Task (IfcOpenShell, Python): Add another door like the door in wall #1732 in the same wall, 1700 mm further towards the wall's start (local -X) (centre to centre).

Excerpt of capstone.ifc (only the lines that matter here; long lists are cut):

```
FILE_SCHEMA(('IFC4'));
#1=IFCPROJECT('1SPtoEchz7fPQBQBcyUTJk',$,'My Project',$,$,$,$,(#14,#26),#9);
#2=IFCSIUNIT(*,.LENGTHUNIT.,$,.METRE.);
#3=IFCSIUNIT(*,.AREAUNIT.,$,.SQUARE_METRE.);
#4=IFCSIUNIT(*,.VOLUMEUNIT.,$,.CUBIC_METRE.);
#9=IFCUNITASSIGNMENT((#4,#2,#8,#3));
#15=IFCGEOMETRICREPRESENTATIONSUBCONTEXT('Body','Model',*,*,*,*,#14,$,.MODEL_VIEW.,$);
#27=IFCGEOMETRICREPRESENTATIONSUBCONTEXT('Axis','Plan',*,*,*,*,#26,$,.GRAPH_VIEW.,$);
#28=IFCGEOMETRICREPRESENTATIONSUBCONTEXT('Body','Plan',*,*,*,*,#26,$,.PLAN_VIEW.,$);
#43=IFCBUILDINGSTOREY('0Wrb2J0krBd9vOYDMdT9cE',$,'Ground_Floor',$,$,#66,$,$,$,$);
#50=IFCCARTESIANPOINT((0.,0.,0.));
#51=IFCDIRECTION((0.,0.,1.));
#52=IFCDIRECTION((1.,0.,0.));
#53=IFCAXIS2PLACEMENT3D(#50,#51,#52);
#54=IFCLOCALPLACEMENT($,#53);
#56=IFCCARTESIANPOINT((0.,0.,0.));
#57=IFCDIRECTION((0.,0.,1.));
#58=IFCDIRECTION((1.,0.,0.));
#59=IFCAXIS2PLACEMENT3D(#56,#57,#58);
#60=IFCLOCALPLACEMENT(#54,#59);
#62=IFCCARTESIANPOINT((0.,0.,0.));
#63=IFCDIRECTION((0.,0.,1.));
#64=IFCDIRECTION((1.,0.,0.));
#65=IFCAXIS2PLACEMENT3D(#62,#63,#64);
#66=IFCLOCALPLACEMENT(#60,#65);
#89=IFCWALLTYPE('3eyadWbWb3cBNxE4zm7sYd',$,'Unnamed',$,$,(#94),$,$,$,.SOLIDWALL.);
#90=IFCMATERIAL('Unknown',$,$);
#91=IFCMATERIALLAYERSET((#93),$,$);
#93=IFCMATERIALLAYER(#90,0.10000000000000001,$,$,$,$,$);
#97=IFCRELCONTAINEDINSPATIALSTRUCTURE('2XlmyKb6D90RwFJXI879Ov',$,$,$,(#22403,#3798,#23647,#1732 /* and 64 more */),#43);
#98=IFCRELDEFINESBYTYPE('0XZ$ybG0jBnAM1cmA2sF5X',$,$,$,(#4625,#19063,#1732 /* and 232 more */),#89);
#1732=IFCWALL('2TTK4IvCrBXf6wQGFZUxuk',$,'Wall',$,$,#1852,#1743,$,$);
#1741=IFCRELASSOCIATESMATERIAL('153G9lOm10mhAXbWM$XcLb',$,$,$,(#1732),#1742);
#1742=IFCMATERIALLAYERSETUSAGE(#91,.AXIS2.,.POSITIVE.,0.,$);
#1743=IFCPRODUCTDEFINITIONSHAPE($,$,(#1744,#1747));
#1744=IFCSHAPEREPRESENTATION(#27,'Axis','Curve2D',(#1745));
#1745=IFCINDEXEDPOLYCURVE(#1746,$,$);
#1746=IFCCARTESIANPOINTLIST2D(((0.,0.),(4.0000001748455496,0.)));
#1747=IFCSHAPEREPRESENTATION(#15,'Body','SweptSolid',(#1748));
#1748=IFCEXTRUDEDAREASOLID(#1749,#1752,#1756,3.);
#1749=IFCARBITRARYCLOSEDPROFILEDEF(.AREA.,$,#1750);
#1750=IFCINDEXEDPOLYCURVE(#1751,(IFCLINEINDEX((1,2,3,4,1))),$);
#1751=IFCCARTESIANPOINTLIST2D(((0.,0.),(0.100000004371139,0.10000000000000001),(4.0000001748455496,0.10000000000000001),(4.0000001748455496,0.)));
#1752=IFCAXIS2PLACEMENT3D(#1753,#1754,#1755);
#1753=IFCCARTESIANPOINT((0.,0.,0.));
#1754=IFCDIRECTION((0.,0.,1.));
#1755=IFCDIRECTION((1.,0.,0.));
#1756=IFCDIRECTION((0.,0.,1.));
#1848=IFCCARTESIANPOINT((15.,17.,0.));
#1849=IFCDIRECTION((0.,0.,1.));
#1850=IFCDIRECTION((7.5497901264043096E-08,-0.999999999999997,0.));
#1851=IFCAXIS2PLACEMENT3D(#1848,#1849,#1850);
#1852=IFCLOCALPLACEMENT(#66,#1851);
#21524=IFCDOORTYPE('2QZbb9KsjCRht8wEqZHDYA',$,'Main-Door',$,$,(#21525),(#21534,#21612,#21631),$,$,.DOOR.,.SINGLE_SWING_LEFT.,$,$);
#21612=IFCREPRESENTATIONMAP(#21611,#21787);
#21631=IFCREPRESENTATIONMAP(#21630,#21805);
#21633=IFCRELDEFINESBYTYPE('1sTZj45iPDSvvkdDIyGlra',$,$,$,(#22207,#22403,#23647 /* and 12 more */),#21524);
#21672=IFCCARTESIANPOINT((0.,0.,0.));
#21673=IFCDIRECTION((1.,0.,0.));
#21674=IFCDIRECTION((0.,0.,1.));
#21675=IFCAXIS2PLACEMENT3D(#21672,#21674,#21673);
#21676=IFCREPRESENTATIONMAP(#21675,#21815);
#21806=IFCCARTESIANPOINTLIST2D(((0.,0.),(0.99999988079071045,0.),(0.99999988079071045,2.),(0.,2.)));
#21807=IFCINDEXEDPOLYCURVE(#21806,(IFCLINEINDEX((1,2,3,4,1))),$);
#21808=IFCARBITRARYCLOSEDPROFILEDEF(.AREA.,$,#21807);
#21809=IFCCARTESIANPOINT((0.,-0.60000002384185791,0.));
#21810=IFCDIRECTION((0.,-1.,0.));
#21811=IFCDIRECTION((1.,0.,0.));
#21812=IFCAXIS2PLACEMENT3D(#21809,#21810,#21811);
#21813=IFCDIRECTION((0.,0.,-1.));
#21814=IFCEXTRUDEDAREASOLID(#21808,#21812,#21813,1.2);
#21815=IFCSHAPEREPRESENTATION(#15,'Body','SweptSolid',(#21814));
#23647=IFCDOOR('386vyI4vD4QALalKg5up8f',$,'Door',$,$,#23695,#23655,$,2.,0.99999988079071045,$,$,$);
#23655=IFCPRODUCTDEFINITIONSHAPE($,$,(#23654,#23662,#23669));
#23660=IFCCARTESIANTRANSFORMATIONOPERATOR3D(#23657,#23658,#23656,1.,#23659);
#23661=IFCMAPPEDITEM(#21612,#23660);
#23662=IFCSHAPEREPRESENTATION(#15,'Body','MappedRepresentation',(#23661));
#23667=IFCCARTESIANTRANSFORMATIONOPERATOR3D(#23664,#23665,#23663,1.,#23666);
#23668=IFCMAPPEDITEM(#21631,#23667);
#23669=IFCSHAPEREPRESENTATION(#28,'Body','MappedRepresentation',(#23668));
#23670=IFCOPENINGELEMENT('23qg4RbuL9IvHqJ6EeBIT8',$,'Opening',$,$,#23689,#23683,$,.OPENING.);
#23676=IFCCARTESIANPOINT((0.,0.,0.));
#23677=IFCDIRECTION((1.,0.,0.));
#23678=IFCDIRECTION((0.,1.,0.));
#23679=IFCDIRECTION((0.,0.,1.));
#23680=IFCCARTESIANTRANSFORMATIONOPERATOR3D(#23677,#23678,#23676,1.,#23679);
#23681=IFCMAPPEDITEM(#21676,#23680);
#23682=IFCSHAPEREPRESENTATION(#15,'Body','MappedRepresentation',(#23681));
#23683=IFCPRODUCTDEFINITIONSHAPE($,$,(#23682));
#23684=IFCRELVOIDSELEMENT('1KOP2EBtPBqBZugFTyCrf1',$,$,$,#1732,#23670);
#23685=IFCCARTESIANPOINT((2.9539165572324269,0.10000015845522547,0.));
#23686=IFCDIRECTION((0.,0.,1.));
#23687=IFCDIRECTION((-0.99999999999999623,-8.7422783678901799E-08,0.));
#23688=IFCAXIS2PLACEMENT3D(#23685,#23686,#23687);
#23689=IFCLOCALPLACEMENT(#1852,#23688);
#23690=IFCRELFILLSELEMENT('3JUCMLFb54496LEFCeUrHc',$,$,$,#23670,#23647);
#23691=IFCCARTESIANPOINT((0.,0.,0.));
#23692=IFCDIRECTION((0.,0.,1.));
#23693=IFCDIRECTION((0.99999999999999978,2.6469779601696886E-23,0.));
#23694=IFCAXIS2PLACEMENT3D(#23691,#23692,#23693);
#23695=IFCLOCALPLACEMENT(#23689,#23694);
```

```python
import ifcopenshell
import ifcopenshell.api.feature
import ifcopenshell.api.geometry
import ifcopenshell.api.root
import ifcopenshell.geom
import ifcopenshell.util.element
import ifcopenshell.util.placement
import ifcopenshell.util.shape
import ifcopenshell.util.unit

model = ifcopenshell.open("capstone.ifc")
unit_scale = ifcopenshell.util.unit.calculate_unit_scale(model)
settings = ifcopenshell.geom.settings()


def volume(element):
    """Net volume in cubic metres, openings subtracted."""
    shape = ifcopenshell.geom.create_shape(settings, element)
    return ifcopenshell.util.shape.get_volume(shape.geometry)


door = model.by_guid("386vyI4vD4QALalKg5up8f")
opening = door.FillsVoids[0].RelatingOpeningElement
wall = opening.VoidsElements[0].RelatingBuildingElement
before = volume(wall)
shift = ifcopenshell.util.placement.get_local_placement(wall.ObjectPlacement)[:3, 0] * -1.7 / unit_scale

# copy_class copies the void relationship, type, container and properties, but no geometry.
new_opening = ifcopenshell.api.root.copy_class(model, product=opening)
new_opening.Representation = ifcopenshell.util.element.copy_deep(
    model, opening.Representation, exclude=["IfcGeometricRepresentationContext", "IfcRepresentationMap"]
)
new_door = ifcopenshell.api.root.copy_class(model, product=door)
new_door.Representation = ifcopenshell.util.element.copy_deep(
    model, door.Representation, exclude=["IfcGeometricRepresentationContext", "IfcRepresentationMap"]
)
ifcopenshell.api.feature.add_filling(model, opening=new_opening, element=new_door)

for old, new in ((opening, new_opening), (door, new_door)):
    matrix = ifcopenshell.util.placement.get_local_placement(old.ObjectPlacement)
    matrix[:3, 3] += shift
    ifcopenshell.api.geometry.edit_object_placement(model, product=new, matrix=matrix, is_si=False)

after = volume(wall)

print(f"wall volume {before:.3f} -> {after:.3f} m3")

model.write("capstone_updated.ifc")
```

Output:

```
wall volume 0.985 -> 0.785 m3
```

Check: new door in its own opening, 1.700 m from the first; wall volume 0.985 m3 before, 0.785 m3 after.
